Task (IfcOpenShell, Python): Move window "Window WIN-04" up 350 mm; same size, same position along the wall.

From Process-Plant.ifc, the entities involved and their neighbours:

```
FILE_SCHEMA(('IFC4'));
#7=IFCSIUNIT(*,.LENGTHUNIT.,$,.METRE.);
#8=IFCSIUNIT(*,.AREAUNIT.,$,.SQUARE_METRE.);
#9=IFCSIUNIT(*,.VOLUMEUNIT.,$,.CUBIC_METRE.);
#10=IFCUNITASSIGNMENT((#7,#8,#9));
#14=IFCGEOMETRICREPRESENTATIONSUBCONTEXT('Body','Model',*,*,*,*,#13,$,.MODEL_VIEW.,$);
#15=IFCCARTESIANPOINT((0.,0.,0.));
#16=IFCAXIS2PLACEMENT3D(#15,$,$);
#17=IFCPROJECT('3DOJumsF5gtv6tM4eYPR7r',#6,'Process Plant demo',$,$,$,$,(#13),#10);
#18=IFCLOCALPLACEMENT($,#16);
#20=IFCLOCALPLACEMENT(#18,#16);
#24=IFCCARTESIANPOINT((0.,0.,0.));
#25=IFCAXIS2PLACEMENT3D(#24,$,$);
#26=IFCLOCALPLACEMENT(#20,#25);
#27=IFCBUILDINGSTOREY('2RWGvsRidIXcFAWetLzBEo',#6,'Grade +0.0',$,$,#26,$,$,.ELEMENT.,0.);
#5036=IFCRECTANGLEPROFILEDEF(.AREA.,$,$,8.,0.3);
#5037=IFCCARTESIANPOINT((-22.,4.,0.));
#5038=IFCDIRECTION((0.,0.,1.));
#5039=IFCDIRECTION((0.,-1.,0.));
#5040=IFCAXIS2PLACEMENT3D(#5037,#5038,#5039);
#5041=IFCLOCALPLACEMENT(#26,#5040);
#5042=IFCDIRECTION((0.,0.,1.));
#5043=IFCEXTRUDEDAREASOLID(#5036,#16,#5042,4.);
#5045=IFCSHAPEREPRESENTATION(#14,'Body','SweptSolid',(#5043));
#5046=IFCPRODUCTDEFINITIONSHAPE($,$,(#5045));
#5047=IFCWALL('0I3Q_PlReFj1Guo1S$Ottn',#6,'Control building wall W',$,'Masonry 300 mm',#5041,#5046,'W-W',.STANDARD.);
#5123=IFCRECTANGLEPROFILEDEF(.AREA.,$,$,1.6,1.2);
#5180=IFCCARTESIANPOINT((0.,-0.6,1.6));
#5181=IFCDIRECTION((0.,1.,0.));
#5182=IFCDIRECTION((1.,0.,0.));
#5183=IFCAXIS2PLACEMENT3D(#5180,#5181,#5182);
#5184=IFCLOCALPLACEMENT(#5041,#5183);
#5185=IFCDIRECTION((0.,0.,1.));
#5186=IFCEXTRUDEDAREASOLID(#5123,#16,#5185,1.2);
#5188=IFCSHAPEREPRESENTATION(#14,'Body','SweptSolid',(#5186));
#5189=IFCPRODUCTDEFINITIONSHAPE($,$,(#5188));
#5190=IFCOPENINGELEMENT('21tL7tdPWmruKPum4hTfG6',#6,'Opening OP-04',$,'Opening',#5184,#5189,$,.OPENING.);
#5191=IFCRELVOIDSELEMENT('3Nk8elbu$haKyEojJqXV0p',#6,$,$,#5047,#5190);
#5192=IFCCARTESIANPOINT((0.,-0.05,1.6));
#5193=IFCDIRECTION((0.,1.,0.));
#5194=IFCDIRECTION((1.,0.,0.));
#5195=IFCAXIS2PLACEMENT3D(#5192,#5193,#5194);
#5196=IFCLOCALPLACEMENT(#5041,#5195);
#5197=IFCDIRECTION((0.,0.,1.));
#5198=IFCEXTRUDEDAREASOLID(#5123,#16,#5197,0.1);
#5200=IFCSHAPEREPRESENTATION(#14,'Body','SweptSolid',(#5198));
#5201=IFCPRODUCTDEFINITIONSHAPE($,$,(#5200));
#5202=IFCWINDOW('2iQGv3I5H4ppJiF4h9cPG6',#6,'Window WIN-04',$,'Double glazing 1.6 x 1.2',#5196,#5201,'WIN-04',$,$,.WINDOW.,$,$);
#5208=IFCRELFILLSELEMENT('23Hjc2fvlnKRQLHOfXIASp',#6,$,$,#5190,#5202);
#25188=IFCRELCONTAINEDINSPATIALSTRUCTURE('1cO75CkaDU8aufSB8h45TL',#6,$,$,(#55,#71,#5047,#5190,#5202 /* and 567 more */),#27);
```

```python
import numpy as np
import ifcopenshell
import ifcopenshell.api.geometry
import ifcopenshell.util.placement
import ifcopenshell.util.unit

model = ifcopenshell.open("Process-Plant.ifc")
unit_scale = ifcopenshell.util.unit.calculate_unit_scale(model)

window = model.by_guid("2iQGv3I5H4ppJiF4h9cPG6")
opening = window.FillsVoids[0].RelatingOpeningElement
dz = 0.35 / unit_scale

shift = np.array([0.0, 0.0, dz])
# The window is not placed relative to its opening, so move both.
for product in (opening, window):
    matrix = ifcopenshell.util.placement.get_local_placement(product.ObjectPlacement)
    matrix[:3, 3] += shift
    ifcopenshell.api.geometry.edit_object_placement(model, product=product, matrix=matrix, is_si=False)

print(f"moved by {dz * unit_scale:+.3f} m")

model.write("Process-Plant_updated.ifc")
```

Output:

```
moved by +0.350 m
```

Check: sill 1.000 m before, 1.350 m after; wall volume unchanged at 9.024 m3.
